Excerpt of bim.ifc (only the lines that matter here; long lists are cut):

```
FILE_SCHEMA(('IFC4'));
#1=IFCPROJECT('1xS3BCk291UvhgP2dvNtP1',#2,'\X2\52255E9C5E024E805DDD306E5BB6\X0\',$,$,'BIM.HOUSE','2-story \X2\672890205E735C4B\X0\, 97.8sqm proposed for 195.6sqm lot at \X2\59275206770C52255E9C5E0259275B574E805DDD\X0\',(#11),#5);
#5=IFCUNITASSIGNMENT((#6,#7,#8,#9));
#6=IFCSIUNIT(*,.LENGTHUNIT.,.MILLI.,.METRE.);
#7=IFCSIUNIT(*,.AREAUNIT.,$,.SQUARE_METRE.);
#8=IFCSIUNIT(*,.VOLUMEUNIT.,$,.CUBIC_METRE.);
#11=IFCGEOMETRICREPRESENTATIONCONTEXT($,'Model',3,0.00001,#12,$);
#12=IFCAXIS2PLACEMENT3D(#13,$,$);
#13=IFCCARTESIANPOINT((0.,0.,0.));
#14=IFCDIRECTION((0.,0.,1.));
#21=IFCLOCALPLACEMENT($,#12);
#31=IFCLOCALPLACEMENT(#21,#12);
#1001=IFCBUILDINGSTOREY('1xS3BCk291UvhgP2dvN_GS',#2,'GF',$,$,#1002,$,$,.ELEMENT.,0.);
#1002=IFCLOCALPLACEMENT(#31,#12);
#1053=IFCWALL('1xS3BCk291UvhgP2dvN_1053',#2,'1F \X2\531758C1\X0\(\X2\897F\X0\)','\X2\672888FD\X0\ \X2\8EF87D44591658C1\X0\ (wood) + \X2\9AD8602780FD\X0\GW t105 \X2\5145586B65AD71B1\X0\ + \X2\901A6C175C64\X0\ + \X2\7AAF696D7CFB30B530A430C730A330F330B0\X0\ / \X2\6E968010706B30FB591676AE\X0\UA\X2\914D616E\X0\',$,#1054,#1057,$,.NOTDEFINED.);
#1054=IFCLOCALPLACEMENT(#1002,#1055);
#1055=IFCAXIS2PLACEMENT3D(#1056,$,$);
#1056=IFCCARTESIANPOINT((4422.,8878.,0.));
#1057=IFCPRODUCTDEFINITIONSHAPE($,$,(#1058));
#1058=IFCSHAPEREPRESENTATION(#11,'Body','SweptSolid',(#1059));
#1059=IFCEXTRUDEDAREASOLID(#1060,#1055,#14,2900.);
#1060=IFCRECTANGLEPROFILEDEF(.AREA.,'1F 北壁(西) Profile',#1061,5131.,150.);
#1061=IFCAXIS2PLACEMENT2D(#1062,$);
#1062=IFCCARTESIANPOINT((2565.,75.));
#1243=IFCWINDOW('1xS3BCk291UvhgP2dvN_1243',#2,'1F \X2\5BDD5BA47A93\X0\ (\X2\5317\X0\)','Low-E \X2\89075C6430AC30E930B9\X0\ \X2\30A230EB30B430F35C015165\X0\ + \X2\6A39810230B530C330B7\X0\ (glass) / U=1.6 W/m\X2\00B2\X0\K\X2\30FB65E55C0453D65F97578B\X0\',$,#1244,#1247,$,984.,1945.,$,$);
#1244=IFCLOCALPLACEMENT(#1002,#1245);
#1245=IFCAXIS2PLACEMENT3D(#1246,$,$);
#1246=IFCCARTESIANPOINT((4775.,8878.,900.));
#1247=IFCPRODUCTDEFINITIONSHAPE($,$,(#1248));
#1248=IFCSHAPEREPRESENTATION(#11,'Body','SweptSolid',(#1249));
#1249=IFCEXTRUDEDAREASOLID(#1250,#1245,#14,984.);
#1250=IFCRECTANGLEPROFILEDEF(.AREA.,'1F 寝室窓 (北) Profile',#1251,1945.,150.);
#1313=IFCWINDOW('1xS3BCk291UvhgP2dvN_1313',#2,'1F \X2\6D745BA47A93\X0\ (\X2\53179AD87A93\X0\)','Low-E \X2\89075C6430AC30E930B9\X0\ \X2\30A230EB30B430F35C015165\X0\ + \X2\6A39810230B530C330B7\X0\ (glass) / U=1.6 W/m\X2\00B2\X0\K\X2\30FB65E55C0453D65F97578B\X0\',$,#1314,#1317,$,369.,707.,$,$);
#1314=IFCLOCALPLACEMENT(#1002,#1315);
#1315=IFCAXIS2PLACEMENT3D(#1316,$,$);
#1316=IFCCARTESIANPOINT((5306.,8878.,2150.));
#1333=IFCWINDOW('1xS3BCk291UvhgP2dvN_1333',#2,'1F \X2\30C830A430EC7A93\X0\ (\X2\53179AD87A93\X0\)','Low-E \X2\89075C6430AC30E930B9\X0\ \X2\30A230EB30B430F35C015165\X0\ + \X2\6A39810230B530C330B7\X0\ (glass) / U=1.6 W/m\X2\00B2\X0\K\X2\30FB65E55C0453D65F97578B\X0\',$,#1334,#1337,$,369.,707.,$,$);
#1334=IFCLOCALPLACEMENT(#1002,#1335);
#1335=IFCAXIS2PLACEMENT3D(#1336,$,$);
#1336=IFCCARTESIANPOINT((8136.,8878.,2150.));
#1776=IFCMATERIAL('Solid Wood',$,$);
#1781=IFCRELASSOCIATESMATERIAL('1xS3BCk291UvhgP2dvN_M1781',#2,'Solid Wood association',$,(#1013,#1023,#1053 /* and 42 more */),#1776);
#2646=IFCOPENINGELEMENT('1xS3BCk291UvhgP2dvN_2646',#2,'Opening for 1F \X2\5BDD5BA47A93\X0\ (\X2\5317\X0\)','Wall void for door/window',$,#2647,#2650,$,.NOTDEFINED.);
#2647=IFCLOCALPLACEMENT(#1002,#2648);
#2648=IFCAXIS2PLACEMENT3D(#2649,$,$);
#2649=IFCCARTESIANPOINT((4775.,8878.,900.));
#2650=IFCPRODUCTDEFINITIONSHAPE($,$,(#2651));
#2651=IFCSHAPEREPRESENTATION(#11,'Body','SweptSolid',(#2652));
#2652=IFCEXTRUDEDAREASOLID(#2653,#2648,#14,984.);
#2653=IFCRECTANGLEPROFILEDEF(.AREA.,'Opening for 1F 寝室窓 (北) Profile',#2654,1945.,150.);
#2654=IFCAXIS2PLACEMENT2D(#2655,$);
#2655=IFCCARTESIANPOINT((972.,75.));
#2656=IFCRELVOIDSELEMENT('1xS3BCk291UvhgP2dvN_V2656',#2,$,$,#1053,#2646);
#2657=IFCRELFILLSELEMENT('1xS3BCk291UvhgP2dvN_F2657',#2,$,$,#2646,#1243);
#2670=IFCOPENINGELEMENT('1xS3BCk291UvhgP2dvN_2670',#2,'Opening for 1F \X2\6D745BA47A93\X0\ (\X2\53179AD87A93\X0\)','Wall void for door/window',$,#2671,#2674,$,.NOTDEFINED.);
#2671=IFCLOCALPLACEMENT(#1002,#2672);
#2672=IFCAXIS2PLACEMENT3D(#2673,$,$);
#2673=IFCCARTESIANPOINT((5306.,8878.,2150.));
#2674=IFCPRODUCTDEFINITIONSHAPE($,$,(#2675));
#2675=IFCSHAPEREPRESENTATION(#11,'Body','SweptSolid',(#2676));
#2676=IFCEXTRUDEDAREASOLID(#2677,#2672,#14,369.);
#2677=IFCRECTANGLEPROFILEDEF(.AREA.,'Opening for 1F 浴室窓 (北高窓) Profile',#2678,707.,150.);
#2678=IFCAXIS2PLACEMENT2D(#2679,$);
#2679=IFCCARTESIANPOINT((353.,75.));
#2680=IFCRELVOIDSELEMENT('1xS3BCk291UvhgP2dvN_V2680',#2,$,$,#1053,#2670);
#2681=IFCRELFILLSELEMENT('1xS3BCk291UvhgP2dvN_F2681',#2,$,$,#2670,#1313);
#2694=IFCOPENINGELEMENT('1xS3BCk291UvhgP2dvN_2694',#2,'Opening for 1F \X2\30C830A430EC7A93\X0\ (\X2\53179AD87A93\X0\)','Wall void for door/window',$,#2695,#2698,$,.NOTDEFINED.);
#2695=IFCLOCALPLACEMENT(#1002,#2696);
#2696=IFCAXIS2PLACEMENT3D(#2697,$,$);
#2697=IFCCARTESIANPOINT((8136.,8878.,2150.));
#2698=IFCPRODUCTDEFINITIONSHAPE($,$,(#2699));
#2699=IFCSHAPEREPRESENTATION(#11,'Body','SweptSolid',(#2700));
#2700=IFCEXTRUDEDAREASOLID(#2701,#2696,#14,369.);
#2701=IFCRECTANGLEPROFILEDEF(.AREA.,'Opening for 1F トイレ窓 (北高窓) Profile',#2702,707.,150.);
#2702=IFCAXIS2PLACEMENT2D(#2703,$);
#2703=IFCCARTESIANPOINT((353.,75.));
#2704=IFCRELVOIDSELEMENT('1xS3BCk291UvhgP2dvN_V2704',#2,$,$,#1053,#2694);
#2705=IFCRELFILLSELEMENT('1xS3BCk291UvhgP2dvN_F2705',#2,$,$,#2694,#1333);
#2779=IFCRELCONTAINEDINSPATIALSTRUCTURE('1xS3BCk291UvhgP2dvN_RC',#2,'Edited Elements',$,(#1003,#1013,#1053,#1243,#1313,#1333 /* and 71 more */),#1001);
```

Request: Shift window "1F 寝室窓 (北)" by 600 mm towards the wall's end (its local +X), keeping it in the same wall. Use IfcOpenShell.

```python
import ifcopenshell
import ifcopenshell.api.geometry
import ifcopenshell.util.placement
import ifcopenshell.util.unit

model = ifcopenshell.open("bim.ifc")
unit_scale = ifcopenshell.util.unit.calculate_unit_scale(model)

window = model.by_guid("1xS3BCk291UvhgP2dvN_1243")
opening = window.FillsVoids[0].RelatingOpeningElement
wall = opening.VoidsElements[0].RelatingBuildingElement

wall_matrix = ifcopenshell.util.placement.get_local_placement(wall.ObjectPlacement)
shift = wall_matrix[:3, 0] * 0.6 / unit_scale
before = ifcopenshell.util.placement.get_local_placement(window.ObjectPlacement)[:3, 3].copy()

# The window is not placed relative to its opening, so move both.
for product in (opening, window):
    matrix = ifcopenshell.util.placement.get_local_placement(product.ObjectPlacement)
    matrix[:3, 3] += shift
    ifcopenshell.api.geometry.edit_object_placement(model, product=product, matrix=matrix, is_si=False)

after = ifcopenshell.util.placement.get_local_placement(window.ObjectPlacement)[:3, 3]
print("window moved by", (after - before).round(3) + 0.0)

model.write("bim_updated.ifc")
```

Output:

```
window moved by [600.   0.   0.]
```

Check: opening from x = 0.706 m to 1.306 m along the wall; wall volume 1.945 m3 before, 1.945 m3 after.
